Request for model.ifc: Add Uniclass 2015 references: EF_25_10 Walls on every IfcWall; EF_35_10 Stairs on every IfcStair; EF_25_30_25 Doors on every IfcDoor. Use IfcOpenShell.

First a look at what the model holds.

```python
import ifcopenshell

model = ifcopenshell.open("model.ifc")
print(model.schema)
print("classifications:", [c.Name for c in model.by_type("IfcClassification")])
for ifc_class in ("IfcDoor", "IfcRoof", "IfcStair", "IfcWall", "IfcWindow"):
    print(ifc_class, len(model.by_type(ifc_class)))
```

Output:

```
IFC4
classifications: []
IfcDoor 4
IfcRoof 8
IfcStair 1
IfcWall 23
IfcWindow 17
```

```python
import ifcopenshell
import ifcopenshell.api.classification

model = ifcopenshell.open("model.ifc")

system = ifcopenshell.api.classification.add_classification(model, classification="Uniclass 2015")

codes = {
    "IfcWall": ("EF_25_10", "Walls"),
    "IfcStair": ("EF_35_10", "Stairs"),
    "IfcDoor": ("EF_25_30_25", "Doors"),
}
for ifc_class, (code, name) in codes.items():
    products = model.by_type(ifc_class)
    ifcopenshell.api.classification.add_reference(
        model, products=products, classification=system, identification=code, name=name
    )
    print(code, len(products))

model.write("model_edited.ifc")
```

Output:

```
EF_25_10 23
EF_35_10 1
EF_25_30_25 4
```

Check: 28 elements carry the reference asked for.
